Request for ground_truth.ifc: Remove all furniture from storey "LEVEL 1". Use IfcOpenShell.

First a look at what the model holds.

```python
import ifcopenshell
import ifcopenshell.util.element

model = ifcopenshell.open("ground_truth.ifc")
print(model.schema)
storey = next(s for s in model.by_type("IfcBuildingStorey") if s.Name == "LEVEL 1")
furniture = [e for e in ifcopenshell.util.element.get_decomposition(storey) if e.is_a("IfcFurnishingElement")]
seen = {}
for e in furniture:
    element_type = ifcopenshell.util.element.get_type(e)
    name = element_type.Name if element_type not in (None, e) else None
    seen[name] = seen.get(name, 0) + 1
for name, count in sorted(seen.items(), key=str):
    print(count, "x", name)
```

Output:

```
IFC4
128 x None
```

```python
import ifcopenshell
import ifcopenshell.api.root
import ifcopenshell.util.element

model = ifcopenshell.open("ground_truth.ifc")

storey = next(s for s in model.by_type("IfcBuildingStorey") if s.Name == "LEVEL 1")
furniture = [e for e in ifcopenshell.util.element.get_decomposition(storey) if e.is_a("IfcFurnishingElement")]

for e in furniture:
    ifcopenshell.api.root.remove_product(model, product=e)
print(len(furniture), "removed")

model.write("ground_truth_v2.ifc")
```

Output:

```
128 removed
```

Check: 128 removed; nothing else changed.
